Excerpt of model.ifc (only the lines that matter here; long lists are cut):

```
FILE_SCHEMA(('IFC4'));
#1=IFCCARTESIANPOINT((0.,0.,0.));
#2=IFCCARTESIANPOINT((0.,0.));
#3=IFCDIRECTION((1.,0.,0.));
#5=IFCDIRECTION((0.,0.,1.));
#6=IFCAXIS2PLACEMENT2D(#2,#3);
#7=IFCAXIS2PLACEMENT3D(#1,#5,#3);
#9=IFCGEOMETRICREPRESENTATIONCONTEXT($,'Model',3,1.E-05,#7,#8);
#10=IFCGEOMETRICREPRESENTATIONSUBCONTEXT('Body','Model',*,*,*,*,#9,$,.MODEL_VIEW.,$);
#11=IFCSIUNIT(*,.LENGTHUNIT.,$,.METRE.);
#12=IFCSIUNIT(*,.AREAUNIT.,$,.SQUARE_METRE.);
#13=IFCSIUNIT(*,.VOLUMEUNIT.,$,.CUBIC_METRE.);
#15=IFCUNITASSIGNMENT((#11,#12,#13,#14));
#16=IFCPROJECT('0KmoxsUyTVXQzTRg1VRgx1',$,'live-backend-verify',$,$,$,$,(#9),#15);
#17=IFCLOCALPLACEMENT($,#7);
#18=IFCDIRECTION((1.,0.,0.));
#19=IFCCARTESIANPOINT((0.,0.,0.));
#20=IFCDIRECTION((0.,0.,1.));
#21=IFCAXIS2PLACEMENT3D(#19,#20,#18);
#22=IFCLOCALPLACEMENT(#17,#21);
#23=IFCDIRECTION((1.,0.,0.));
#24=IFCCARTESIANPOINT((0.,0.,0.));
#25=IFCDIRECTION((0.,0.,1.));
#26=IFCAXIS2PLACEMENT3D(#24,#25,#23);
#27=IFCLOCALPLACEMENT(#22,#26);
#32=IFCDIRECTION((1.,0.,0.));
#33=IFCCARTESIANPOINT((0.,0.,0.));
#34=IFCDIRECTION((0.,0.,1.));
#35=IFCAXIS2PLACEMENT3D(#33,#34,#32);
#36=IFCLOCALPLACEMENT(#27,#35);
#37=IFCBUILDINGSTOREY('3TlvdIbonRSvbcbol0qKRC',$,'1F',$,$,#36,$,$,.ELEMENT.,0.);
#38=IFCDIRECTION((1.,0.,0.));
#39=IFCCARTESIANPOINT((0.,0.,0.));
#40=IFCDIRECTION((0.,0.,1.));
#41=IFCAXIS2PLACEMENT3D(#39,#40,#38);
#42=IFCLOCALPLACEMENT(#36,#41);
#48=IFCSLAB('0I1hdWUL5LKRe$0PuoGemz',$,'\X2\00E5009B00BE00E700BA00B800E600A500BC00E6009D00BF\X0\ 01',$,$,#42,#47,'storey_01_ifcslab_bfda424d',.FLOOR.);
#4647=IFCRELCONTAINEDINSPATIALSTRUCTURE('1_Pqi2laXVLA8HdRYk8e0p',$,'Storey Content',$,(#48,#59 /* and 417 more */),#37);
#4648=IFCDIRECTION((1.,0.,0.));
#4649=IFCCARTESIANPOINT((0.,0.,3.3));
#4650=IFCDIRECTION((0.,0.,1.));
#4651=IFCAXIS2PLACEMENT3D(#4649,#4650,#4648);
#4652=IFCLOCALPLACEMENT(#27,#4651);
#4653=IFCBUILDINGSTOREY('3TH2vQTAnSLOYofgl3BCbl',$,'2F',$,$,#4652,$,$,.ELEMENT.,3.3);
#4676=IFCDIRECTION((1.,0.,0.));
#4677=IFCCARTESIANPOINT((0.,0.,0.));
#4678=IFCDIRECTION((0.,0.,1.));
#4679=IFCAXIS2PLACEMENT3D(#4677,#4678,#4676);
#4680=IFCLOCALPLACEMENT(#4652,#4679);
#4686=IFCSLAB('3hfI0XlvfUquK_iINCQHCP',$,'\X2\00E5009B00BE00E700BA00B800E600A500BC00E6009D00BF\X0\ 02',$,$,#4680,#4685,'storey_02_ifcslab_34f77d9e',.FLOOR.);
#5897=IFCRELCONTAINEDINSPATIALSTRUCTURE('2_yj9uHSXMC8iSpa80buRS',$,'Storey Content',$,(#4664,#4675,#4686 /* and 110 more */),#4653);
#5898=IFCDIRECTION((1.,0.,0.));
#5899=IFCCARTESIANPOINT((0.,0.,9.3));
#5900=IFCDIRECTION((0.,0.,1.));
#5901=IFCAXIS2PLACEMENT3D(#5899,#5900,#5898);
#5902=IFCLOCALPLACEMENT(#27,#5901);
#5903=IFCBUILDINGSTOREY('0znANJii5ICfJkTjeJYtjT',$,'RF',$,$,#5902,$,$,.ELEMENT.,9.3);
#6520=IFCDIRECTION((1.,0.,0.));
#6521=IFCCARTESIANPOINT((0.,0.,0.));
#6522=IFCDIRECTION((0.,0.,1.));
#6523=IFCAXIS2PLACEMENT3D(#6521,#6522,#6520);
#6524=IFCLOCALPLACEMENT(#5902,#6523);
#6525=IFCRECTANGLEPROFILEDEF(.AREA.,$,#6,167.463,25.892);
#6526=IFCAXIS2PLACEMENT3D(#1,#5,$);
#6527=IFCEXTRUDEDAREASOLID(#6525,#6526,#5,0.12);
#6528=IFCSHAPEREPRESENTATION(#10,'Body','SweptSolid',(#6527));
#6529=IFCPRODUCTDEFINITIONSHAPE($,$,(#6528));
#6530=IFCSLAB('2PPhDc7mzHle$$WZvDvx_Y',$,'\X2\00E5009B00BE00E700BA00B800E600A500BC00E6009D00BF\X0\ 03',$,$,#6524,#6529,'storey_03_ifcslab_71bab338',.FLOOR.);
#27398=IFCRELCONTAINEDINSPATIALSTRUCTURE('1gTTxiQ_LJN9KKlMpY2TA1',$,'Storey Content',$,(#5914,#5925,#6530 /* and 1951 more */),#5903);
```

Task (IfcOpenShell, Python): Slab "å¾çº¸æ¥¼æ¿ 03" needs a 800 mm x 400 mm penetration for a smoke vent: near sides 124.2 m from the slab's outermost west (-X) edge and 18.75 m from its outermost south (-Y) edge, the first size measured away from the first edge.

```python
import numpy as np
import ifcopenshell
import ifcopenshell.api.feature
import ifcopenshell.api.geometry
import ifcopenshell.api.root
import ifcopenshell.geom
import ifcopenshell.util.placement
import ifcopenshell.util.representation
import ifcopenshell.util.shape
import ifcopenshell.util.unit

model = ifcopenshell.open("model.ifc")
unit_scale = ifcopenshell.util.unit.calculate_unit_scale(model)
settings = ifcopenshell.geom.settings()


def volume(element):
    """Net volume in cubic metres, openings subtracted."""
    shape = ifcopenshell.geom.create_shape(settings, element)
    return ifcopenshell.util.shape.get_volume(shape.geometry)


slab = model.by_guid("2PPhDc7mzHle$$WZvDvx_Y")
before = volume(slab)

# Extent in the slab's own axes, in metres. The edges named are its -X and -Y sides.
slab_shape = ifcopenshell.geom.create_shape(settings, slab)
vertices = ifcopenshell.util.shape.get_vertices(slab_shape.geometry)
x_min, y_min, bottom = vertices.min(axis=0)
top = vertices[:, 2].max()

opening = ifcopenshell.api.root.create_entity(model, ifc_class="IfcOpeningElement", name="Smoke vent opening", predefined_type="OPENING")
context = ifcopenshell.util.representation.get_context(model, "Model", "Body", "MODEL_VIEW")
width, depth = 0.8, 0.4
outline = [(0.0, 0.0), (width, 0.0), (width, depth), (0.0, depth), (0.0, 0.0)]
# Overshoot both faces by 50 mm so the cut is clean.
shape = ifcopenshell.api.geometry.add_slab_representation(
    model, context=context, depth=top - bottom + 0.1, polyline=outline
)
ifcopenshell.api.geometry.assign_representation(model, product=opening, representation=shape)

matrix = ifcopenshell.util.placement.get_local_placement(slab.ObjectPlacement)
matrix[:, 3] = matrix @ np.append(np.array([x_min + 124.2, y_min + 18.75, bottom - 0.05]) / unit_scale, 1.0)
ifcopenshell.api.geometry.edit_object_placement(model, product=opening, matrix=matrix, is_si=False)
ifcopenshell.api.feature.add_feature(model, feature=opening, element=slab)

after = volume(slab)

print(f"slab volume {before:.3f} -> {after:.3f} m3")

model.write("model_edited.ifc")
```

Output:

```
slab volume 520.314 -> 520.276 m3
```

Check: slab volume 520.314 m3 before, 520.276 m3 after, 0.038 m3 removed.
